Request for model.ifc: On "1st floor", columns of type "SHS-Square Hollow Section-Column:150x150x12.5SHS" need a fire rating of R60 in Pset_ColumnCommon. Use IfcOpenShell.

First a look at what the model holds.

```python
import ifcopenshell
import ifcopenshell.util.element

model = ifcopenshell.open("model.ifc")
print(model.schema)
storey = next(s for s in model.by_type("IfcBuildingStorey") if s.Name == "1st floor")
columns = [e for e in ifcopenshell.util.element.get_decomposition(storey) if e.is_a("IfcColumn")]
seen = {}
for e in columns:
    element_type = ifcopenshell.util.element.get_type(e)
    key = (element_type.Name if element_type != e and element_type else None, ifcopenshell.util.element.get_pset(e, "Pset_ColumnCommon", "FireRating"))
    seen[key] = seen.get(key, 0) + 1
for (name, value), count in sorted(seen.items(), key=str):
    print(count, "x", name, "|", value)
```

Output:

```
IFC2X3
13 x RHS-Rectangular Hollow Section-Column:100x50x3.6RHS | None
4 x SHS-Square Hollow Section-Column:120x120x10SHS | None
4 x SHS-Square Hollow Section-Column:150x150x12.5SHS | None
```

```python
import ifcopenshell
import ifcopenshell.api.pset
import ifcopenshell.util.element

model = ifcopenshell.open("model.ifc")

storey = next(s for s in model.by_type("IfcBuildingStorey") if s.Name == "1st floor")
columns = [e for e in ifcopenshell.util.element.get_decomposition(storey) if e.is_a("IfcColumn")]

count = 0
for e in columns:
    element_type = ifcopenshell.util.element.get_type(e)
    if element_type in (None, e) or element_type.Name != "SHS-Square Hollow Section-Column:150x150x12.5SHS":
        continue
    # add_pset returns the element's existing set when there is one.
    pset = ifcopenshell.api.pset.add_pset(model, product=e, name="Pset_ColumnCommon")
    ifcopenshell.api.pset.edit_pset(model, pset=pset, properties={"FireRating": "R60"})
    count += 1

print(count, "columns updated")

model.write("model-out.ifc")
```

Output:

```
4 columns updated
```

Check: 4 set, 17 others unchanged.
